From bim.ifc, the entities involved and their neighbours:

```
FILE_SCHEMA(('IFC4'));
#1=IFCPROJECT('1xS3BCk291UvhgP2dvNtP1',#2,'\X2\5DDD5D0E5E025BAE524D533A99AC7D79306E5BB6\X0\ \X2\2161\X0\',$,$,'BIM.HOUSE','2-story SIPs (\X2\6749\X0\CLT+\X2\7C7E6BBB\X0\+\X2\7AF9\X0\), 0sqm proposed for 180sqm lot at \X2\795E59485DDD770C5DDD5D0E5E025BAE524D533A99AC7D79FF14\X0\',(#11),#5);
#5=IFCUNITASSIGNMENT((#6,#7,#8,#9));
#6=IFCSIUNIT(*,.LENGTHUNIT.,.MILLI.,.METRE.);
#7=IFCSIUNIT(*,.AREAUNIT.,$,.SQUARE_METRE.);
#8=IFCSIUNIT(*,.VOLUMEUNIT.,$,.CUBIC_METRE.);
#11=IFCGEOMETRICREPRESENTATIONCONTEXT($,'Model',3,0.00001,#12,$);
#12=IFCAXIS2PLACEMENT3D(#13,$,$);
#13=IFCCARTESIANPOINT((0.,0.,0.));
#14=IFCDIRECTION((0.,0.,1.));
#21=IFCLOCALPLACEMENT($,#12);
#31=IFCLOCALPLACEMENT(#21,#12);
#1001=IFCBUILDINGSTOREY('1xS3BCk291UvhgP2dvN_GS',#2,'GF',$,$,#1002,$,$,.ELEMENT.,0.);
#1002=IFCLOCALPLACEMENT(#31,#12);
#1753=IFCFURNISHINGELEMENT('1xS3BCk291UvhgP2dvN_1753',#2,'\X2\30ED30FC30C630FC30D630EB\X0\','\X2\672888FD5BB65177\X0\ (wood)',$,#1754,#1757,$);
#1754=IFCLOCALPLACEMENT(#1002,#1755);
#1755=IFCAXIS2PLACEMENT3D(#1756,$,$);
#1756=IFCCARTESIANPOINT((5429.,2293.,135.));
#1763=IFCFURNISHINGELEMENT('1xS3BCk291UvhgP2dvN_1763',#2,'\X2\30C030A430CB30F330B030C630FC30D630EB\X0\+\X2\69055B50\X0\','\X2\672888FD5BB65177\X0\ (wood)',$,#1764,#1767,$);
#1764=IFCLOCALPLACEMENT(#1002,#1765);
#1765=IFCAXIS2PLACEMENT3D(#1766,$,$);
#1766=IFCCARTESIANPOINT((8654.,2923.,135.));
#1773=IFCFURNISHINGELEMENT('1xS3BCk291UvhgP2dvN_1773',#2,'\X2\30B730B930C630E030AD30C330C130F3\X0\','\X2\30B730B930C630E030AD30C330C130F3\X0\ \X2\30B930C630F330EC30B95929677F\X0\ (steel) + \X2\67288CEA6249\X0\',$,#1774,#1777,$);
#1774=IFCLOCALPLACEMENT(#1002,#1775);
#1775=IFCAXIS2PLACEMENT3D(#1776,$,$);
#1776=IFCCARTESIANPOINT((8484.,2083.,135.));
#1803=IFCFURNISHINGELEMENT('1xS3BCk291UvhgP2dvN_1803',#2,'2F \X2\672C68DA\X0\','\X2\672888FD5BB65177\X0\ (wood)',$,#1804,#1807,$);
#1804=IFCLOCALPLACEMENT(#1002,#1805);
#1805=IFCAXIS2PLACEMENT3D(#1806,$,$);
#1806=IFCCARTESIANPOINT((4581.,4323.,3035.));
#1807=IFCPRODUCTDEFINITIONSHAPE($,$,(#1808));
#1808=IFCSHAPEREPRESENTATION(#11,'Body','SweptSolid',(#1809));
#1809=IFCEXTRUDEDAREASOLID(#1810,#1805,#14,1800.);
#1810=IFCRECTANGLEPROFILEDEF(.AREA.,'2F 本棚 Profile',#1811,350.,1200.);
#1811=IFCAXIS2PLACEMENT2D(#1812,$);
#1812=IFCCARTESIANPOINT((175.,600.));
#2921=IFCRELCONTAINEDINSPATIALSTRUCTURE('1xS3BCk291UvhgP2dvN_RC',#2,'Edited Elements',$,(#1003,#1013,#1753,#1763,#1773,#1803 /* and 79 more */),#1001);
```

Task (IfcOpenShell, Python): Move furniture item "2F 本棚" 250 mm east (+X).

```python
import ifcopenshell
import ifcopenshell.api.geometry
import ifcopenshell.util.placement
import ifcopenshell.util.unit

model = ifcopenshell.open("bim.ifc")
unit_scale = ifcopenshell.util.unit.calculate_unit_scale(model)

item = model.by_guid("1xS3BCk291UvhgP2dvN_1803")
matrix = ifcopenshell.util.placement.get_local_placement(item.ObjectPlacement)
matrix[0, 3] += 0.25 / unit_scale
ifcopenshell.api.geometry.edit_object_placement(model, product=item, matrix=matrix, is_si=False)

print(ifcopenshell.util.placement.get_local_placement(item.ObjectPlacement).round(3) + 0.0)

model.write("bim_rev.ifc")
```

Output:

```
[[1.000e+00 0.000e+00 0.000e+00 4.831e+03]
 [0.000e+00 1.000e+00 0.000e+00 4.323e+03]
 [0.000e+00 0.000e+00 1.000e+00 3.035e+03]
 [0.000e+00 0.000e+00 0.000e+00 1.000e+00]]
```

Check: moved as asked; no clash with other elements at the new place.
